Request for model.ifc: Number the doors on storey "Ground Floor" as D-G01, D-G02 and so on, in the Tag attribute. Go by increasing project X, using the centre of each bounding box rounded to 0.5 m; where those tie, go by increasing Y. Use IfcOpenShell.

First a look at what the model holds.

```python
import ifcopenshell
import ifcopenshell.util.element
import ifcopenshell.util.placement

model = ifcopenshell.open("model.ifc")
print(model.schema)
storey = next(s for s in model.by_type("IfcBuildingStorey") if s.Name == "Ground Floor")
doors = [e for e in ifcopenshell.util.element.get_decomposition(storey) if e.is_a("IfcDoor")]
for e in sorted(doors, key=lambda e: e.id()):
    origin = ifcopenshell.util.placement.get_local_placement(e.ObjectPlacement)[:3, 3]
    print(e.id(), e.Tag, e.Name, origin.round(2) + 0.0, sep=" | ")
```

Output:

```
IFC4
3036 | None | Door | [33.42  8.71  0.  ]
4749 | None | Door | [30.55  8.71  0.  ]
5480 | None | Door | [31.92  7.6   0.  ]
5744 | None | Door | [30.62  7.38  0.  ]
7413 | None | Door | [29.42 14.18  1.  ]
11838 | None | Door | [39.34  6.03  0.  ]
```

```python
import ifcopenshell
import ifcopenshell.geom
import ifcopenshell.util.element
import ifcopenshell.util.shape

model = ifcopenshell.open("model.ifc")
settings = ifcopenshell.geom.settings()
settings.set("use-world-coords", True)


def centre(element):
    shape = ifcopenshell.geom.create_shape(settings, element)
    return ifcopenshell.util.shape.get_bbox_centroid(shape.geometry)


storey = next(s for s in model.by_type("IfcBuildingStorey") if s.Name == "Ground Floor")
doors = [e for e in ifcopenshell.util.element.get_decomposition(storey) if e.is_a("IfcDoor")]

# Insertion points can sit at a corner or the storey origin, so sort by the geometry (in metres).
centres = {e: centre(e) for e in doors}
doors.sort(key=lambda e: (round(centres[e][0] / 0.5), centres[e][1]))

for i, e in enumerate(doors, start=1):
    number = f"D-G{i:02d}"
    e.Tag = number
    print(e.id(), number)

model.write("model_updated.ifc")
```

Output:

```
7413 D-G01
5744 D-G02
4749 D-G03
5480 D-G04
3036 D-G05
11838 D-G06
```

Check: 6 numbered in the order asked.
